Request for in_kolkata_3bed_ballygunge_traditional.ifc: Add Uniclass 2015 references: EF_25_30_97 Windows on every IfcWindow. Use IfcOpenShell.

First a look at what the model holds.

```python
import ifcopenshell

model = ifcopenshell.open("in_kolkata_3bed_ballygunge_traditional.ifc")
print(model.schema)
print("classifications:", [c.Name for c in model.by_type("IfcClassification")])
for ifc_class in ("IfcDoor", "IfcRoof", "IfcStair", "IfcWall", "IfcWindow"):
    print(ifc_class, len(model.by_type(ifc_class)))
```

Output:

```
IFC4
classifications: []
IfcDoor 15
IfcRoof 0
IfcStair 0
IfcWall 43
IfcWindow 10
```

```python
import ifcopenshell
import ifcopenshell.api.classification

model = ifcopenshell.open("in_kolkata_3bed_ballygunge_traditional.ifc")

system = ifcopenshell.api.classification.add_classification(model, classification="Uniclass 2015")

codes = {
    "IfcWindow": ("EF_25_30_97", "Windows"),
}
for ifc_class, (code, name) in codes.items():
    products = model.by_type(ifc_class)
    ifcopenshell.api.classification.add_reference(
        model, products=products, classification=system, identification=code, name=name
    )
    print(code, len(products))

model.write("in_kolkata_3bed_ballygunge_traditional_rev.ifc")
```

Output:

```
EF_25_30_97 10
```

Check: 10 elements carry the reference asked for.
